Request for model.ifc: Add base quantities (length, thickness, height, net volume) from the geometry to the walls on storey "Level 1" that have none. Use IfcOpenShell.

First a look at what the model holds.

```python
import ifcopenshell
import ifcopenshell.util.element
import ifcopenshell.util.unit

model = ifcopenshell.open("model.ifc")
print(model.schema)
for unit_type in ("LENGTHUNIT", "AREAUNIT", "VOLUMEUNIT"):
    print(unit_type, ifcopenshell.util.unit.calculate_unit_scale(model, unit_type))
storey = next(s for s in model.by_type("IfcBuildingStorey") if s.Name == "Level 1")
walls = [e for e in ifcopenshell.util.element.get_decomposition(storey) if e.is_a("IfcWall")]
for e in sorted(walls, key=lambda e: e.id()):
    print(e.id(), e.is_a(), e.Name, list(ifcopenshell.util.element.get_psets(e, qtos_only=True)), sep=" | ")
```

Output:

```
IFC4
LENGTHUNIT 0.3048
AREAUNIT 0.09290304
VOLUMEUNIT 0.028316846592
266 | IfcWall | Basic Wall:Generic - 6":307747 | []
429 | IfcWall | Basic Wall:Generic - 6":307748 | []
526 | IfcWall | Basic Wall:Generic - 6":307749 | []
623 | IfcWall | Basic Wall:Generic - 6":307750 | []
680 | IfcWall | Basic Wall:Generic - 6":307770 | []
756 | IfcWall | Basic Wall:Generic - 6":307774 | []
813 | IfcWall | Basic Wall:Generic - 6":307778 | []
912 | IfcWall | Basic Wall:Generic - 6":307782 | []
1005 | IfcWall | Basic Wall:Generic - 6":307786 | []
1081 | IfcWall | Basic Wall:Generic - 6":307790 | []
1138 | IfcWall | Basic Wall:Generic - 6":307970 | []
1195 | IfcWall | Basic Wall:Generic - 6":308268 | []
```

```python
import ifcopenshell
import ifcopenshell.api.pset
import ifcopenshell.geom
import ifcopenshell.util.element
import ifcopenshell.util.shape
import ifcopenshell.util.unit

model = ifcopenshell.open("model.ifc")
unit_scale = ifcopenshell.util.unit.calculate_unit_scale(model)
volume_scale = ifcopenshell.util.unit.calculate_unit_scale(model, "VOLUMEUNIT")
settings = ifcopenshell.geom.settings()

storey = next(s for s in model.by_type("IfcBuildingStorey") if s.Name == "Level 1")
walls = [e for e in ifcopenshell.util.element.get_decomposition(storey) if e.is_a("IfcWall")]

for e in sorted(walls, key=lambda e: e.id()):
    if ifcopenshell.util.element.get_psets(e, qtos_only=True, should_inherit=False):
        continue
    # Geometry comes back in metres, in the element's own axes.
    shape = ifcopenshell.geom.create_shape(settings, e)
    values = {
        "Length": ifcopenshell.util.shape.get_x(shape.geometry) / unit_scale,
        "Width": ifcopenshell.util.shape.get_y(shape.geometry) / unit_scale,
        "Height": ifcopenshell.util.shape.get_z(shape.geometry) / unit_scale,
        "NetVolume": ifcopenshell.util.shape.get_volume(shape.geometry) / volume_scale,
    }
    qto = ifcopenshell.api.pset.add_qto(model, product=e, name="Qto_WallBaseQuantities")
    ifcopenshell.api.pset.edit_qto(model, qto=qto, properties=values)
    print(e.id(), {k: round(v, 3) for k, v in values.items()})

model.write("model_v2.ifc")
```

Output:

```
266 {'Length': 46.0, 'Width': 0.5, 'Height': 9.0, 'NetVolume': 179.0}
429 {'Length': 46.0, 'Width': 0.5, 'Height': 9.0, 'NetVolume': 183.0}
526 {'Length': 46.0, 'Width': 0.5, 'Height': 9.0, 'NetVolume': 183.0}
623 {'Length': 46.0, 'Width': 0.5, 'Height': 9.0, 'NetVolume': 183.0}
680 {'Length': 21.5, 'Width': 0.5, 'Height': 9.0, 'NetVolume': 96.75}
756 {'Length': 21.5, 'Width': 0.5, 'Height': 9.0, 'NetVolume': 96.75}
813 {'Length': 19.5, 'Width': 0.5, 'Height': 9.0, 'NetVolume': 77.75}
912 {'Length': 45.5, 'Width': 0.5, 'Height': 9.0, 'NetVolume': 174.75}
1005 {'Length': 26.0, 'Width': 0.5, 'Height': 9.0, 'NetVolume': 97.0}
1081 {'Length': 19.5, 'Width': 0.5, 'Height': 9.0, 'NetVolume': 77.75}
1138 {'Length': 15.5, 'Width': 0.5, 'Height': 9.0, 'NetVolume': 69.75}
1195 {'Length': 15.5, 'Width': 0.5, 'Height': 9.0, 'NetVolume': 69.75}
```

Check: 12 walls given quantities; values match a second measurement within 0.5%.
